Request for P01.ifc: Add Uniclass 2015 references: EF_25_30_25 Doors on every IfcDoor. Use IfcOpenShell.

First a look at what the model holds.

```python
import ifcopenshell

model = ifcopenshell.open("P01.ifc")
print(model.schema)
print("classifications:", [c.Name for c in model.by_type("IfcClassification")])
for ifc_class in ("IfcDoor", "IfcRoof", "IfcStair", "IfcWall", "IfcWindow"):
    print(ifc_class, len(model.by_type(ifc_class)))
```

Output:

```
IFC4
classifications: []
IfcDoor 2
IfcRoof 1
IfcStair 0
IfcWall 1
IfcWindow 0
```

```python
import ifcopenshell
import ifcopenshell.api.classification

model = ifcopenshell.open("P01.ifc")

system = ifcopenshell.api.classification.add_classification(model, classification="Uniclass 2015")

codes = {
    "IfcDoor": ("EF_25_30_25", "Doors"),
}
for ifc_class, (code, name) in codes.items():
    products = model.by_type(ifc_class)
    ifcopenshell.api.classification.add_reference(
        model, products=products, classification=system, identification=code, name=name
    )
    print(code, len(products))

model.write("P01_rev.ifc")
```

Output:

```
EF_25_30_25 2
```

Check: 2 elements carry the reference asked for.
